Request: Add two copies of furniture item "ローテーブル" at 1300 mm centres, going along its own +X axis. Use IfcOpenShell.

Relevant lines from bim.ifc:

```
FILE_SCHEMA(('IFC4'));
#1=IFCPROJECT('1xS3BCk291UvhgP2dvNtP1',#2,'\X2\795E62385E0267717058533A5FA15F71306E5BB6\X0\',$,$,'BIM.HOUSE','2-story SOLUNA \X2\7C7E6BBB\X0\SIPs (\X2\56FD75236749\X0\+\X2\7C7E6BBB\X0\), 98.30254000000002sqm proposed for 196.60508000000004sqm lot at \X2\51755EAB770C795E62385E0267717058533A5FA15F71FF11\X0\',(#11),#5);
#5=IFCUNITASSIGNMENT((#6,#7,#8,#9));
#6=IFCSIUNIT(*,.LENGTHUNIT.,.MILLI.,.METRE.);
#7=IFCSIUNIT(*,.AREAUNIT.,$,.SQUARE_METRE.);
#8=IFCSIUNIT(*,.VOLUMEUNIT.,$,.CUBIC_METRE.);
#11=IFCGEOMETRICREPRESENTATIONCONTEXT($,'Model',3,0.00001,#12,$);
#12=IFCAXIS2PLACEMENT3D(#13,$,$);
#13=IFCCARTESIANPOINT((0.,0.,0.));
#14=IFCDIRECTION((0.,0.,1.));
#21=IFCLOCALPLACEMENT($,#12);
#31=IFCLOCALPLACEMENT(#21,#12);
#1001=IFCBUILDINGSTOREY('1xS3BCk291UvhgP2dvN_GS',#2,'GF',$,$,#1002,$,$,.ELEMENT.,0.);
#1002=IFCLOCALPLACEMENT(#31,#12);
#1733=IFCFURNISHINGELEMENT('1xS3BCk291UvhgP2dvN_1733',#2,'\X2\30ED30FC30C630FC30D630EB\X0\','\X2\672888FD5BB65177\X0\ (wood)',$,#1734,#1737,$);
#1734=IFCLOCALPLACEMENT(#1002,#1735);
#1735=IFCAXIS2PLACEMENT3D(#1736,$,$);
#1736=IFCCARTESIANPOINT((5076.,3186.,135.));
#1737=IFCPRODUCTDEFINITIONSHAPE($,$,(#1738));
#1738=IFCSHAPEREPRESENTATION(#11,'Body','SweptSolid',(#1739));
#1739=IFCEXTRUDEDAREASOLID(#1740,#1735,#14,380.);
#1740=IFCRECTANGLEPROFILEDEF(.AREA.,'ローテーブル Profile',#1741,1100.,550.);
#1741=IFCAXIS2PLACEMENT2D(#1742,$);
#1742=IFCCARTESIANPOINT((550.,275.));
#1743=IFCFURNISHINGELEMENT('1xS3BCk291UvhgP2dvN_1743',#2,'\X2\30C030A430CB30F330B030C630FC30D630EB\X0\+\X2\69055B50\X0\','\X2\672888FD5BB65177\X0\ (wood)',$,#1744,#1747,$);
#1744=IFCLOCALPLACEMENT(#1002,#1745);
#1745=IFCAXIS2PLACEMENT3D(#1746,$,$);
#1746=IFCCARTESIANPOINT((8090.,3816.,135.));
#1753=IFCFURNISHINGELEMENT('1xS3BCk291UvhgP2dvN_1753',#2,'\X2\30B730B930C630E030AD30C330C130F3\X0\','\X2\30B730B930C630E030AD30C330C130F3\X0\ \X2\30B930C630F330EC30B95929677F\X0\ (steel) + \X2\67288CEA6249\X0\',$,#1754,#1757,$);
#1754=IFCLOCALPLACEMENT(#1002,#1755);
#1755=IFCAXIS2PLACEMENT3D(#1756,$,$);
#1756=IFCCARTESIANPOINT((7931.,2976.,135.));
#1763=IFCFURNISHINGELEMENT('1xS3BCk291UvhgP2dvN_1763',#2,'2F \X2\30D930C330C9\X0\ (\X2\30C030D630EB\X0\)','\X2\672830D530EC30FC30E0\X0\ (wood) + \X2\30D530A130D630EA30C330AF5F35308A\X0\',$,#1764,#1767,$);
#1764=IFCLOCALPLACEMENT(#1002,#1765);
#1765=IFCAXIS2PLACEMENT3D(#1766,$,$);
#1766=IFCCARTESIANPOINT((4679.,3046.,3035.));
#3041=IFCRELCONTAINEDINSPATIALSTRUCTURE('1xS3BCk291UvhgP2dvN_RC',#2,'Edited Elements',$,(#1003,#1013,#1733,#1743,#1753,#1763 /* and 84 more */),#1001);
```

```python
import ifcopenshell
import ifcopenshell.api.geometry
import ifcopenshell.api.root
import ifcopenshell.util.element
import ifcopenshell.util.placement

model = ifcopenshell.open("bim.ifc")


def reuse_history(source, copy):
    """copy_class also copies each property set's owner history, people and application; keep the originals."""
    for rel in copy.IsDefinedBy:
        if rel.is_a("IfcRelDefinesByProperties") and (history := rel.RelatingPropertyDefinition.OwnerHistory):
            rel.RelatingPropertyDefinition.OwnerHistory = source.OwnerHistory
            ifcopenshell.util.element.remove_deep2(model, history)


source = model.by_guid("1xS3BCk291UvhgP2dvN_1733")
base = ifcopenshell.util.placement.get_local_placement(source.ObjectPlacement)
step = base[:3, 0] * 1300.0

for i in range(1, 3):
    copy = ifcopenshell.api.root.copy_class(model, product=source)
    copy.Representation = ifcopenshell.util.element.copy_deep(
        model, source.Representation, exclude=["IfcGeometricRepresentationContext", "IfcRepresentationMap"]
    )
    reuse_history(source, copy)
    matrix = base.copy()
    matrix[:3, 3] += i * step
    print("added at", matrix[:3, 3].round(3) + 0.0)
    ifcopenshell.api.geometry.edit_object_placement(model, product=copy, matrix=matrix, is_si=False)

model.write("bim_rev.ifc")
```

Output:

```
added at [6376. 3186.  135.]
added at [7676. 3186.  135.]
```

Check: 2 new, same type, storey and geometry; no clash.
